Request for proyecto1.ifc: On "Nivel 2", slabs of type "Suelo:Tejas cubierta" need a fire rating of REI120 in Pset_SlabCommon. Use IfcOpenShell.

First a look at what the model holds.

```python
import ifcopenshell
import ifcopenshell.util.element

model = ifcopenshell.open("proyecto1.ifc")
print(model.schema)
storey = next(s for s in model.by_type("IfcBuildingStorey") if s.Name == "Nivel 2")
slabs = [e for e in ifcopenshell.util.element.get_decomposition(storey) if e.is_a("IfcSlab")]
seen = {}
for e in slabs:
    element_type = ifcopenshell.util.element.get_type(e)
    key = (element_type.Name if element_type != e and element_type else None, ifcopenshell.util.element.get_pset(e, "Pset_SlabCommon", "FireRating"))
    seen[key] = seen.get(key, 0) + 1
for (name, value), count in sorted(seen.items(), key=str):
    print(count, "x", name, "|", value)
```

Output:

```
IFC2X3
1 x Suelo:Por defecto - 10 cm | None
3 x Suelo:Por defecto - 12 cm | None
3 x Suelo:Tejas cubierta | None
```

```python
import ifcopenshell
import ifcopenshell.api.pset
import ifcopenshell.util.element

model = ifcopenshell.open("proyecto1.ifc")

storey = next(s for s in model.by_type("IfcBuildingStorey") if s.Name == "Nivel 2")
slabs = [e for e in ifcopenshell.util.element.get_decomposition(storey) if e.is_a("IfcSlab")]

count = 0
for e in slabs:
    element_type = ifcopenshell.util.element.get_type(e)
    if element_type in (None, e) or element_type.Name != "Suelo:Tejas cubierta":
        continue
    # add_pset returns the element's existing set when there is one.
    pset = ifcopenshell.api.pset.add_pset(model, product=e, name="Pset_SlabCommon")
    ifcopenshell.api.pset.edit_pset(model, pset=pset, properties={"FireRating": "REI120"})
    count += 1

print(count, "slabs updated")

model.write("proyecto1_updated.ifc")
```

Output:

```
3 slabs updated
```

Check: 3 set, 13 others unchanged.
